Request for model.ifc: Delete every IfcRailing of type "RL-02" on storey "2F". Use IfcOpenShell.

First a look at what the model holds.

```python
import ifcopenshell
import ifcopenshell.util.element

model = ifcopenshell.open("model.ifc")
print(model.schema)
storey = next(s for s in model.by_type("IfcBuildingStorey") if s.Name == "2F")
railings = [e for e in ifcopenshell.util.element.get_decomposition(storey) if e.is_a("IfcRailing")]
seen = {}
for e in railings:
    element_type = ifcopenshell.util.element.get_type(e)
    name = element_type.Name if element_type not in (None, e) else None
    seen[name] = seen.get(name, 0) + 1
for name, count in sorted(seen.items(), key=str):
    print(count, "x", name)
```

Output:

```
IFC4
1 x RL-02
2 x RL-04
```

```python
import ifcopenshell
import ifcopenshell.api.root
import ifcopenshell.util.element

model = ifcopenshell.open("model.ifc")

storey = next(s for s in model.by_type("IfcBuildingStorey") if s.Name == "2F")
railings = [e for e in ifcopenshell.util.element.get_decomposition(storey) if e.is_a("IfcRailing")]
targets = [e for e in railings if (t := ifcopenshell.util.element.get_type(e)) not in (None, e) and t.Name == "RL-02"]

for e in targets:
    ifcopenshell.api.root.remove_product(model, product=e)
print(len(targets), "removed")

model.write("model_v2.ifc")
```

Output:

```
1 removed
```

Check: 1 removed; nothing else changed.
